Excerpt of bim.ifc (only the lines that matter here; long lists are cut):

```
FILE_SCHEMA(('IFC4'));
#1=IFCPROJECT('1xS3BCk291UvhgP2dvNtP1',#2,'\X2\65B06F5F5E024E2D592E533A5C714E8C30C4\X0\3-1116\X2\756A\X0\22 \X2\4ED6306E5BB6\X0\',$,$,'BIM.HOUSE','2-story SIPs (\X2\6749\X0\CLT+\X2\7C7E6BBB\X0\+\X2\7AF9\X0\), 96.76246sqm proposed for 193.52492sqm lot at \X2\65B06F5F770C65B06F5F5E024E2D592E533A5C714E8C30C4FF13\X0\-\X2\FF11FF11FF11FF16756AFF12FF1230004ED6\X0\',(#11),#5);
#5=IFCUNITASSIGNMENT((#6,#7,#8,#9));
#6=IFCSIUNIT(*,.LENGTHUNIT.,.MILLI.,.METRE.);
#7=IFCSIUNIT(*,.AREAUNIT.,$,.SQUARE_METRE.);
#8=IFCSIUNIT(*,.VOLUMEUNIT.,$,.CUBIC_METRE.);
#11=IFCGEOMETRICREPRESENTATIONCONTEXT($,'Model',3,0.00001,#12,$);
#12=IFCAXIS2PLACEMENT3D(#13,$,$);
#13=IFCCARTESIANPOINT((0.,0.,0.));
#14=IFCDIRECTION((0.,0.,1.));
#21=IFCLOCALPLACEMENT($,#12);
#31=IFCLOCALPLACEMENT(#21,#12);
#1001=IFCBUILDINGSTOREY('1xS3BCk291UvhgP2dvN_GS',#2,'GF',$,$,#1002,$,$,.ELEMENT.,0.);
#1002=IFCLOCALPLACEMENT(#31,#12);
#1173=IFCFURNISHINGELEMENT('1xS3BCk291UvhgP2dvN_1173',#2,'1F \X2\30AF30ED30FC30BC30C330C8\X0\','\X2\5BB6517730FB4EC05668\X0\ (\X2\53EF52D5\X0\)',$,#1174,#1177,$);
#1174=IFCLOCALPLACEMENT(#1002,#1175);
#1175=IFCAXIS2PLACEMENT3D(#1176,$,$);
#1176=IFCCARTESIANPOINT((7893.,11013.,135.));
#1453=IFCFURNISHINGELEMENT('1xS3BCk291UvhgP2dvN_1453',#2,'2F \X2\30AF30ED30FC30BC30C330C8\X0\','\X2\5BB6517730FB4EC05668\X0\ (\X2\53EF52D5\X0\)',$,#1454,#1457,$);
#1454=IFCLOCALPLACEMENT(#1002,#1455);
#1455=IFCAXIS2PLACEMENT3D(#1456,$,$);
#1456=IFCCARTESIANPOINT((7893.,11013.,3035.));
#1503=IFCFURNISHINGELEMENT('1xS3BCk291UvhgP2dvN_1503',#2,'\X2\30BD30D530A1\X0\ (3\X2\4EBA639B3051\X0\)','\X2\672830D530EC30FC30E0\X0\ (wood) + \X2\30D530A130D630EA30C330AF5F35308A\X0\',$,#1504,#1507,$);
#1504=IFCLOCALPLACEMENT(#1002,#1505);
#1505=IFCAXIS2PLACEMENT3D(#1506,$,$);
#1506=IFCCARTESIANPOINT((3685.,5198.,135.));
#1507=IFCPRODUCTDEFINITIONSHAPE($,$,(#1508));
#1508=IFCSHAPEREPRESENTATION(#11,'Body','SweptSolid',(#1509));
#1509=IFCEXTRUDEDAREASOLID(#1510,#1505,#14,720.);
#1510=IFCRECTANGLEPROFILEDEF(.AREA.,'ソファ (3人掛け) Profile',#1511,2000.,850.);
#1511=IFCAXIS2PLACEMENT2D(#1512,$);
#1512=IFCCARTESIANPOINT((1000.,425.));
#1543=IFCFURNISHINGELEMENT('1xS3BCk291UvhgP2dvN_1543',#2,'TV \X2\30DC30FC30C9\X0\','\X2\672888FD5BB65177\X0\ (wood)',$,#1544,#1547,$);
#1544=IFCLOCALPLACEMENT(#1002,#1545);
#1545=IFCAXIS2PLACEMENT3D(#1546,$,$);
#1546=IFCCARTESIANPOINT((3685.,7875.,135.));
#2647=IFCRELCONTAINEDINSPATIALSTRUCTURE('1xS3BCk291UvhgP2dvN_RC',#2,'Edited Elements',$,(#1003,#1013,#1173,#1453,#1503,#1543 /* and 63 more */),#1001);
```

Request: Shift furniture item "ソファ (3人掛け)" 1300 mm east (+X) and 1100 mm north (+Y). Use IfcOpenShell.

```python
import ifcopenshell
import ifcopenshell.api.geometry
import ifcopenshell.util.placement
import ifcopenshell.util.unit

model = ifcopenshell.open("bim.ifc")
unit_scale = ifcopenshell.util.unit.calculate_unit_scale(model)

item = model.by_id(1503)
matrix = ifcopenshell.util.placement.get_local_placement(item.ObjectPlacement)
matrix[0, 3] += 1.3 / unit_scale
matrix[1, 3] += 1.1 / unit_scale
ifcopenshell.api.geometry.edit_object_placement(model, product=item, matrix=matrix, is_si=False)

print(ifcopenshell.util.placement.get_local_placement(item.ObjectPlacement).round(3) + 0.0)

model.write("bim_edited.ifc")
```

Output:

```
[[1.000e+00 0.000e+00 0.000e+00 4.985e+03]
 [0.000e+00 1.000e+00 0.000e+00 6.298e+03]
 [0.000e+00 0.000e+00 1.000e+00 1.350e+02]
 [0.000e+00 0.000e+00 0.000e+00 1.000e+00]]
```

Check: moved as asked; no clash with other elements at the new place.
